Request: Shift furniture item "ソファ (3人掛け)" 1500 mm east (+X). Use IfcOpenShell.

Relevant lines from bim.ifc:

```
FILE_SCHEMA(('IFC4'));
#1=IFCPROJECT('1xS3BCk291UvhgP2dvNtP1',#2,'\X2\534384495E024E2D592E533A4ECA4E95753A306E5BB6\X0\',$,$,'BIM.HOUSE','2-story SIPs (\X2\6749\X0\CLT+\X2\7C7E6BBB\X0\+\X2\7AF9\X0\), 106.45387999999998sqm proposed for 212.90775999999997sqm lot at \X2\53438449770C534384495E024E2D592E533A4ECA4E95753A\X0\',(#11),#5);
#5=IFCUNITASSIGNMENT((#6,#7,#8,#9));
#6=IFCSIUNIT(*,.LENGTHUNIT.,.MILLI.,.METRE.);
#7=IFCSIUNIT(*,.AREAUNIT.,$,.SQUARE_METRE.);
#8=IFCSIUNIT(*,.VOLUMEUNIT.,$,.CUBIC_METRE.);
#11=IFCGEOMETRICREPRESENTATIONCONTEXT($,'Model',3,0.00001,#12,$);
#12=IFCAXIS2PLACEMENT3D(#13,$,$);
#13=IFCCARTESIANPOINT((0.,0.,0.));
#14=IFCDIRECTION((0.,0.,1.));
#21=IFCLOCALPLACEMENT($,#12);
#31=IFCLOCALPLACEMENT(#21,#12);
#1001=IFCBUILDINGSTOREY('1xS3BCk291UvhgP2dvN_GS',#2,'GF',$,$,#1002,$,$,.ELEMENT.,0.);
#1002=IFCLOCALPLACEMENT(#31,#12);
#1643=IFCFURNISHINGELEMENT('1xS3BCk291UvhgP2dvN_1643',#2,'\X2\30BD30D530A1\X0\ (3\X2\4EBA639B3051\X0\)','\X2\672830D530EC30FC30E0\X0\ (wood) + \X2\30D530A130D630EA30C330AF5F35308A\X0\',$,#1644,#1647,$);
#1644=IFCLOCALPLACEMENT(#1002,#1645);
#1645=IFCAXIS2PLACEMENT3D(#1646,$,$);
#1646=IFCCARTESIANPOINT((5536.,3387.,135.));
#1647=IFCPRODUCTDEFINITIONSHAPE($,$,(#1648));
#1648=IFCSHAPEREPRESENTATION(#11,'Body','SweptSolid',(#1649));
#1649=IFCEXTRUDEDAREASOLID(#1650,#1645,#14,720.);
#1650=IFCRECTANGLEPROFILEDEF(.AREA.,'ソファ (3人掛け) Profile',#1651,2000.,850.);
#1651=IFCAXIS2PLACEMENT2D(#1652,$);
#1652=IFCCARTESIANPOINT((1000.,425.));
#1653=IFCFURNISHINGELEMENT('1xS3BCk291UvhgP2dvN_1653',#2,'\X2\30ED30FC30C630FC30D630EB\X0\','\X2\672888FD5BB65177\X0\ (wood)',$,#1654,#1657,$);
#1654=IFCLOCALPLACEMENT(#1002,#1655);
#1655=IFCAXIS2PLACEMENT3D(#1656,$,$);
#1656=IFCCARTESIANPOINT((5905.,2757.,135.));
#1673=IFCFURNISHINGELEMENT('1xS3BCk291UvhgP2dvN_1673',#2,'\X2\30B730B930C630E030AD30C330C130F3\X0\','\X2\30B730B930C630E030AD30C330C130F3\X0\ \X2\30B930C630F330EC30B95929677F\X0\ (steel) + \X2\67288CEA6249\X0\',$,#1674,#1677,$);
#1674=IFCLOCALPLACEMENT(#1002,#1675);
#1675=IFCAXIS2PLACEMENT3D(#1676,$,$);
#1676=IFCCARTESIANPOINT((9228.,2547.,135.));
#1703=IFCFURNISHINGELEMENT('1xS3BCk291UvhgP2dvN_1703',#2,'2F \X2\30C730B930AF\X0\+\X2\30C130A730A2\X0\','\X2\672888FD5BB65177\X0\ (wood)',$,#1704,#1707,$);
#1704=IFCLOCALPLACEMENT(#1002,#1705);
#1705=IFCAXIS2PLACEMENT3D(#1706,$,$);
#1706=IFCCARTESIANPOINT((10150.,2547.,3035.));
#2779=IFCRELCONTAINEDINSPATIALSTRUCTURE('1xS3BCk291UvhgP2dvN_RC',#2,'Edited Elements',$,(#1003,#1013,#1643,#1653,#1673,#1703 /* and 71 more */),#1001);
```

```python
import ifcopenshell
import ifcopenshell.api.geometry
import ifcopenshell.util.placement

model = ifcopenshell.open("bim.ifc")

item = model.by_guid("1xS3BCk291UvhgP2dvN_1643")
matrix = ifcopenshell.util.placement.get_local_placement(item.ObjectPlacement)
matrix[0, 3] += 1500.0
ifcopenshell.api.geometry.edit_object_placement(model, product=item, matrix=matrix, is_si=False)

print(ifcopenshell.util.placement.get_local_placement(item.ObjectPlacement).round(3) + 0.0)

model.write("bim_v2.ifc")
```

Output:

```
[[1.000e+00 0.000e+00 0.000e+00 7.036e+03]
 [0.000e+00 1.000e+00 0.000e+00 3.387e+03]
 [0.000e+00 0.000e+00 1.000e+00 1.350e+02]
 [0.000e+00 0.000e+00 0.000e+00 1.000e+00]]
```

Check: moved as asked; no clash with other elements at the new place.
